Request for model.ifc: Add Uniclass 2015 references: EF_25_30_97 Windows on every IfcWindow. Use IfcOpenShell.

First a look at what the model holds.

```python
import ifcopenshell

model = ifcopenshell.open("model.ifc")
print(model.schema)
print("classifications:", [c.Name for c in model.by_type("IfcClassification")])
for ifc_class in ("IfcDoor", "IfcRoof", "IfcStair", "IfcWall", "IfcWindow"):
    print(ifc_class, len(model.by_type(ifc_class)))
```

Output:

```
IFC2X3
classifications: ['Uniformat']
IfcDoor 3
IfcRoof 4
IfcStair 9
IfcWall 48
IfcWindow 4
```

```python
import ifcopenshell
import ifcopenshell.api.classification

model = ifcopenshell.open("model.ifc")

# IFC2X3 requires Source and Edition and has no link from the project to the system.
system = model.create_entity("IfcClassification", Source="NBS", Edition="2015", Name="Uniclass 2015")

codes = {
    "IfcWindow": ("EF_25_30_97", "Windows"),
}
for ifc_class, (code, name) in codes.items():
    products = model.by_type(ifc_class)
    ifcopenshell.api.classification.add_reference(
        model, products=products, classification=system, identification=code, name=name
    )
    print(code, len(products))

model.write("model-out.ifc")
```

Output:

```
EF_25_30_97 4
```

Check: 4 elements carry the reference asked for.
